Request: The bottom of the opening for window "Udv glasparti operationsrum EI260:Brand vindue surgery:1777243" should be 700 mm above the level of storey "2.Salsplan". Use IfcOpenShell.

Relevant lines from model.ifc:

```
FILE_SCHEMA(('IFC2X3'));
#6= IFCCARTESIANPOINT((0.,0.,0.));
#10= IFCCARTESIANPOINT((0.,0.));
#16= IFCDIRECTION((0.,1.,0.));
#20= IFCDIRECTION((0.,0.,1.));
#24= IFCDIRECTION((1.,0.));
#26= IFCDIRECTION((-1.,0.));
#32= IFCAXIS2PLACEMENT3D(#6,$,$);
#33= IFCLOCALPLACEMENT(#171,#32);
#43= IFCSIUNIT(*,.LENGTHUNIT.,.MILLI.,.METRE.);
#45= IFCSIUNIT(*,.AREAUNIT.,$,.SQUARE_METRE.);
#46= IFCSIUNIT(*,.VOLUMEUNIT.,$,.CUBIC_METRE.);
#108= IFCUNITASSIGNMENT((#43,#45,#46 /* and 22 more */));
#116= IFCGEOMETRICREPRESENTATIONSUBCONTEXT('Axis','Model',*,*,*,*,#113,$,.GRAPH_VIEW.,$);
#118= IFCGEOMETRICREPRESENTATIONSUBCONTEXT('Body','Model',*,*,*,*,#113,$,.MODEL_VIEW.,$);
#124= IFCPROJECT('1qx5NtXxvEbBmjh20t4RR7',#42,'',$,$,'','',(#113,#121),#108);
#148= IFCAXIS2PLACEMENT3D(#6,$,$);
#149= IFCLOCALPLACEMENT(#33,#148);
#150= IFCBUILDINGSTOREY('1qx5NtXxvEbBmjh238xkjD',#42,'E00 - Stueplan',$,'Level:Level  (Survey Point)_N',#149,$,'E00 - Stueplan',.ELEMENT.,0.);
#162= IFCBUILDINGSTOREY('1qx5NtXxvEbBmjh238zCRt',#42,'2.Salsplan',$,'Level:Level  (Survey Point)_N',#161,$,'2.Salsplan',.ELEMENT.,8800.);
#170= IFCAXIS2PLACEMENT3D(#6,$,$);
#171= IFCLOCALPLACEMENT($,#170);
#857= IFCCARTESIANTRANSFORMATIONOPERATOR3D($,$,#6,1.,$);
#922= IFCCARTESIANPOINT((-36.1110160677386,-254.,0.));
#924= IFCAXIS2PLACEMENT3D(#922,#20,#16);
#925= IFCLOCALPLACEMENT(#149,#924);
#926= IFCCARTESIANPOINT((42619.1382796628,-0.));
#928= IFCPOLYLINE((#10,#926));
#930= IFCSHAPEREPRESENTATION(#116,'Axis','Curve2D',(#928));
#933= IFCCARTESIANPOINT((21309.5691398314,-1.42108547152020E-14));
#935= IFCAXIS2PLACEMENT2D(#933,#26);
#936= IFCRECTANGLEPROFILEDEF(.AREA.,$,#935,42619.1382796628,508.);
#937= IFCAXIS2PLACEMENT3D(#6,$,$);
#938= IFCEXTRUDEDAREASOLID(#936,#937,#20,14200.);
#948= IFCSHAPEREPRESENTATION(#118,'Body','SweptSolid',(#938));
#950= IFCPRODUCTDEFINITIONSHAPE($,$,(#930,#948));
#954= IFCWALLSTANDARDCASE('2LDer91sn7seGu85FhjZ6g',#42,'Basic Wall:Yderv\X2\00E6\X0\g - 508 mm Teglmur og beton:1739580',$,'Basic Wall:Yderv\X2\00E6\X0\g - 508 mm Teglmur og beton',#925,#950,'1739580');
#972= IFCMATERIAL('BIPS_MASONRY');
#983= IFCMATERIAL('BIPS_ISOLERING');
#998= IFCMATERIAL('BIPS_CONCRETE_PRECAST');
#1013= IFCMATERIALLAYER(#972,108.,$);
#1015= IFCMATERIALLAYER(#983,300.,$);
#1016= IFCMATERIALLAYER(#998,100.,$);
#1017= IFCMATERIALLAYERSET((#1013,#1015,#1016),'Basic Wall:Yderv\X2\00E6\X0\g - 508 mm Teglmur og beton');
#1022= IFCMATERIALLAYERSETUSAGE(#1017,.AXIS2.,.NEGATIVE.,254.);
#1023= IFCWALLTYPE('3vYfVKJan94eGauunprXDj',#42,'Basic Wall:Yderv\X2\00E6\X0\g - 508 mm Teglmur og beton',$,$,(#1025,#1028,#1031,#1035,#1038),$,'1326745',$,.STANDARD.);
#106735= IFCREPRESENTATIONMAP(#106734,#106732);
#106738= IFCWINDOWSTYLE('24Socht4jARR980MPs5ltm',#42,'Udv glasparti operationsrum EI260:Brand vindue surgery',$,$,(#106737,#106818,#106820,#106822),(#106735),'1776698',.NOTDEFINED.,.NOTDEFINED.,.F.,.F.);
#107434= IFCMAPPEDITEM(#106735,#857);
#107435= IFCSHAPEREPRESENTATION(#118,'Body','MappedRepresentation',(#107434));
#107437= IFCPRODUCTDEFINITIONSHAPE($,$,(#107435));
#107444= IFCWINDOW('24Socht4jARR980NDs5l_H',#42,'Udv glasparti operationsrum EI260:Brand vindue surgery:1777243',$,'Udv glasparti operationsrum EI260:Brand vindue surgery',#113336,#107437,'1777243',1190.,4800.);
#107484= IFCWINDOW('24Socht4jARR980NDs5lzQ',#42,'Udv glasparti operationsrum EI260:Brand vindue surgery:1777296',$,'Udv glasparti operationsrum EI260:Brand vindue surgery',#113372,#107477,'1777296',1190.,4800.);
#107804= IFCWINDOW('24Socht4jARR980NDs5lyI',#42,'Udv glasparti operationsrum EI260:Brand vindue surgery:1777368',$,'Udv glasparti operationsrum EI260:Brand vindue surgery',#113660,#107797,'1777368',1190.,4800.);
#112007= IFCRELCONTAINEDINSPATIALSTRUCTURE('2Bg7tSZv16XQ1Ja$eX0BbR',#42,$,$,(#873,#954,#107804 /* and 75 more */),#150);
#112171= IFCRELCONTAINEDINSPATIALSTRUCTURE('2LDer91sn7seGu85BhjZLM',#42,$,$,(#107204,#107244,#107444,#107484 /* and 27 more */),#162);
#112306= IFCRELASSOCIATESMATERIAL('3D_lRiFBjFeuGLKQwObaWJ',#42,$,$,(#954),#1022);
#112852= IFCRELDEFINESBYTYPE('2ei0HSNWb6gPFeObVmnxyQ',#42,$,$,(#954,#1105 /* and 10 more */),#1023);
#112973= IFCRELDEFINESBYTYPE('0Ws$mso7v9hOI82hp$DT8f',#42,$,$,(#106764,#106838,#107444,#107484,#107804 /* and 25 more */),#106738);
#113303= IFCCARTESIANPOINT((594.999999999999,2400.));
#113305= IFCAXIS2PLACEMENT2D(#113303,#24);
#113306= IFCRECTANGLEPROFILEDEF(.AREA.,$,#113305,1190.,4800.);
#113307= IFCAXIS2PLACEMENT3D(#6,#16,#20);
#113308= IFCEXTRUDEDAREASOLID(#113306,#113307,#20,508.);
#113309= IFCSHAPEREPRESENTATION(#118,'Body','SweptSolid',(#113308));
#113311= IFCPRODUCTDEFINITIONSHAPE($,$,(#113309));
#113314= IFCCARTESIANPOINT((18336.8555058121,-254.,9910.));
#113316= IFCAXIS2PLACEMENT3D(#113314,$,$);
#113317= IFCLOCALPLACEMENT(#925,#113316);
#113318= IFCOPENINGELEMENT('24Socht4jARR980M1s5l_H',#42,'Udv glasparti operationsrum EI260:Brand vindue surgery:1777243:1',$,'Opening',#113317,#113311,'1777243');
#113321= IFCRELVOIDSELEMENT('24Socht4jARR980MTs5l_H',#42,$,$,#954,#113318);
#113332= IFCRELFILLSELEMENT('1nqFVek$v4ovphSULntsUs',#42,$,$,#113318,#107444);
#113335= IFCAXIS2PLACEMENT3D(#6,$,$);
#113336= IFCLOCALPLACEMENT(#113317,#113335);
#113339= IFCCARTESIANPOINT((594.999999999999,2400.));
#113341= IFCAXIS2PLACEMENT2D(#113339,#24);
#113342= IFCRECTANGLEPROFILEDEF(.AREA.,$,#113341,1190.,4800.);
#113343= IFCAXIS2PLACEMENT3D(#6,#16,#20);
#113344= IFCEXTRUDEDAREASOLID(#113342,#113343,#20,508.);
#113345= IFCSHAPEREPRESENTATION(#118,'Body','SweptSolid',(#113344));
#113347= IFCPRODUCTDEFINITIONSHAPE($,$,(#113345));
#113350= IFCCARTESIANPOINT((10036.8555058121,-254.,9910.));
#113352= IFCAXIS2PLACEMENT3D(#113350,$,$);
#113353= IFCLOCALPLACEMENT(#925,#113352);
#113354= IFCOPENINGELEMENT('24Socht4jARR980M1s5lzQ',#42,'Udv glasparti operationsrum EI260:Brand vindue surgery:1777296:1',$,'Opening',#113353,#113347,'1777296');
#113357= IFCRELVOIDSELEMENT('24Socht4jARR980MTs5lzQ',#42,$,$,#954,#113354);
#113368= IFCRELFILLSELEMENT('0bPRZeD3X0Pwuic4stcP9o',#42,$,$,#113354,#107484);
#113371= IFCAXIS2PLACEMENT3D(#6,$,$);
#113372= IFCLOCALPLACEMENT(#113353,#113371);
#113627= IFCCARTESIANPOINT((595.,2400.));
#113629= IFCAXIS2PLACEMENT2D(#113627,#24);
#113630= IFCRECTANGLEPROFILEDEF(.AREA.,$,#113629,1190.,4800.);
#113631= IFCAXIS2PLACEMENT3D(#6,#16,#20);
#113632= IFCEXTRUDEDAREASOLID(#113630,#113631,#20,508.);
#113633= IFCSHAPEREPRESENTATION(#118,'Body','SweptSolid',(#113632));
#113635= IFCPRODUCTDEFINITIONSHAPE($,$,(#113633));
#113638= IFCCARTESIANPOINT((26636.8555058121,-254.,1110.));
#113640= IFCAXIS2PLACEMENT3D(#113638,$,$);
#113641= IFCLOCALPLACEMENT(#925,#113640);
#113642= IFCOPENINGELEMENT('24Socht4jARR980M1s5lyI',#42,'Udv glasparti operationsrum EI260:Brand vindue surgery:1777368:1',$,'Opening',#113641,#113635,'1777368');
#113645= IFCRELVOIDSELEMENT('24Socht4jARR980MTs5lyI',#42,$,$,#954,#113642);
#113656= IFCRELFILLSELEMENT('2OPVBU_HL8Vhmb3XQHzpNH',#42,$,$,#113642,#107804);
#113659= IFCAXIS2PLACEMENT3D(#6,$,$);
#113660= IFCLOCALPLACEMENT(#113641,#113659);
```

```python
import numpy as np
import ifcopenshell
import ifcopenshell.api.geometry
import ifcopenshell.geom
import ifcopenshell.util.element
import ifcopenshell.util.placement
import ifcopenshell.util.shape
import ifcopenshell.util.unit

model = ifcopenshell.open("model.ifc")
unit_scale = ifcopenshell.util.unit.calculate_unit_scale(model)

window = model.by_id(107444)
opening = window.FillsVoids[0].RelatingOpeningElement
storey = ifcopenshell.util.element.get_container(window, ifc_class="IfcBuildingStorey")
level = ifcopenshell.util.placement.get_local_placement(storey.ObjectPlacement)[2, 3]

# The opening's origin need not be at the sill, so measure its lowest point.
shape = ifcopenshell.geom.create_shape(ifcopenshell.geom.settings(), opening)
bottom = ifcopenshell.util.shape.get_shape_bottom_elevation(shape, shape.geometry) / unit_scale
dz = level + 0.7 / unit_scale - bottom

shift = np.array([0.0, 0.0, dz])
# The window is placed relative to its opening, so it follows when the opening moves.
matrix = ifcopenshell.util.placement.get_local_placement(opening.ObjectPlacement)
matrix[:3, 3] += shift
ifcopenshell.api.geometry.edit_object_placement(
    model, product=opening, matrix=matrix, is_si=False, should_transform_children=True
)

print(f"moved by {dz * unit_scale:+.3f} m")

model.write("model-out.ifc")
```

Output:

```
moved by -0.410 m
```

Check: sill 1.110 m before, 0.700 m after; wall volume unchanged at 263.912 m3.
